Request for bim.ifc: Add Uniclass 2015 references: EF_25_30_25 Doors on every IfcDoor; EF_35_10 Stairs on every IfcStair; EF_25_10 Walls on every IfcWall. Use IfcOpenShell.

First a look at what the model holds.

```python
import ifcopenshell

model = ifcopenshell.open("bim.ifc")
print(model.schema)
print("classifications:", [c.Name for c in model.by_type("IfcClassification")])
for ifc_class in ("IfcDoor", "IfcRoof", "IfcStair", "IfcWall", "IfcWindow"):
    print(ifc_class, len(model.by_type(ifc_class)))
```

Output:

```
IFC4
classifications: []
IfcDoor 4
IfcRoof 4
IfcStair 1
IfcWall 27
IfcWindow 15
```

```python
import ifcopenshell
import ifcopenshell.api.classification

model = ifcopenshell.open("bim.ifc")

system = ifcopenshell.api.classification.add_classification(model, classification="Uniclass 2015")

codes = {
    "IfcDoor": ("EF_25_30_25", "Doors"),
    "IfcStair": ("EF_35_10", "Stairs"),
    "IfcWall": ("EF_25_10", "Walls"),
}
for ifc_class, (code, name) in codes.items():
    products = model.by_type(ifc_class)
    ifcopenshell.api.classification.add_reference(
        model, products=products, classification=system, identification=code, name=name
    )
    print(code, len(products))

model.write("bim_v2.ifc")
```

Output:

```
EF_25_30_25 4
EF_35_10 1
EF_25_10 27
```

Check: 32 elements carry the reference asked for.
